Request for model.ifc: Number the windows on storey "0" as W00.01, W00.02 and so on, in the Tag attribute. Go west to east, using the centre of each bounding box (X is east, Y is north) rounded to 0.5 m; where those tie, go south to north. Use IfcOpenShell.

First a look at what the model holds.

```python
import ifcopenshell
import ifcopenshell.util.element
import ifcopenshell.util.placement

model = ifcopenshell.open("model.ifc")
print(model.schema)
storey = next(s for s in model.by_type("IfcBuildingStorey") if s.Name == "0")
windows = [e for e in ifcopenshell.util.element.get_decomposition(storey) if e.is_a("IfcWindow")]
for e in sorted(windows, key=lambda e: e.id()):
    origin = ifcopenshell.util.placement.get_local_placement(e.ObjectPlacement)[:3, 3]
    print(e.id(), e.Tag, e.Name, origin.round(2) + 0.0, sep=" | ")
```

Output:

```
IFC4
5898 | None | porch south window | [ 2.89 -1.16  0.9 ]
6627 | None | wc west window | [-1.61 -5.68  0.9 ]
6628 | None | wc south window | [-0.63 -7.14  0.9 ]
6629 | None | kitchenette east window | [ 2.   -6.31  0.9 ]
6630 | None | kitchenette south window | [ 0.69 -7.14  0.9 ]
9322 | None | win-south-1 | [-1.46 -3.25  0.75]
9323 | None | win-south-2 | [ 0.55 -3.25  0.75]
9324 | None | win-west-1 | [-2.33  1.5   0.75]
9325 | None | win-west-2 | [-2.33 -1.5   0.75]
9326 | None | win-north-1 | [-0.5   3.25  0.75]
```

```python
import ifcopenshell
import ifcopenshell.geom
import ifcopenshell.util.element
import ifcopenshell.util.shape

model = ifcopenshell.open("model.ifc")
settings = ifcopenshell.geom.settings()
settings.set("use-world-coords", True)


def centre(element):
    shape = ifcopenshell.geom.create_shape(settings, element)
    return ifcopenshell.util.shape.get_bbox_centroid(shape.geometry)


storey = next(s for s in model.by_type("IfcBuildingStorey") if s.Name == "0")
windows = [e for e in ifcopenshell.util.element.get_decomposition(storey) if e.is_a("IfcWindow")]

# Insertion points can sit at a corner or the storey origin, so sort by the geometry (in metres).
centres = {e: centre(e) for e in windows}
windows.sort(key=lambda e: (round(centres[e][0] / 0.5), centres[e][1]))

for i, e in enumerate(windows, start=1):
    number = f"W00.{i:02d}"
    e.Tag = number
    print(e.id(), number)

model.write("model_v2.ifc")
```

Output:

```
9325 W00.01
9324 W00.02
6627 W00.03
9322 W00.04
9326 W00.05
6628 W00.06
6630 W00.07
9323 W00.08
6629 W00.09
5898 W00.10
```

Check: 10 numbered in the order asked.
